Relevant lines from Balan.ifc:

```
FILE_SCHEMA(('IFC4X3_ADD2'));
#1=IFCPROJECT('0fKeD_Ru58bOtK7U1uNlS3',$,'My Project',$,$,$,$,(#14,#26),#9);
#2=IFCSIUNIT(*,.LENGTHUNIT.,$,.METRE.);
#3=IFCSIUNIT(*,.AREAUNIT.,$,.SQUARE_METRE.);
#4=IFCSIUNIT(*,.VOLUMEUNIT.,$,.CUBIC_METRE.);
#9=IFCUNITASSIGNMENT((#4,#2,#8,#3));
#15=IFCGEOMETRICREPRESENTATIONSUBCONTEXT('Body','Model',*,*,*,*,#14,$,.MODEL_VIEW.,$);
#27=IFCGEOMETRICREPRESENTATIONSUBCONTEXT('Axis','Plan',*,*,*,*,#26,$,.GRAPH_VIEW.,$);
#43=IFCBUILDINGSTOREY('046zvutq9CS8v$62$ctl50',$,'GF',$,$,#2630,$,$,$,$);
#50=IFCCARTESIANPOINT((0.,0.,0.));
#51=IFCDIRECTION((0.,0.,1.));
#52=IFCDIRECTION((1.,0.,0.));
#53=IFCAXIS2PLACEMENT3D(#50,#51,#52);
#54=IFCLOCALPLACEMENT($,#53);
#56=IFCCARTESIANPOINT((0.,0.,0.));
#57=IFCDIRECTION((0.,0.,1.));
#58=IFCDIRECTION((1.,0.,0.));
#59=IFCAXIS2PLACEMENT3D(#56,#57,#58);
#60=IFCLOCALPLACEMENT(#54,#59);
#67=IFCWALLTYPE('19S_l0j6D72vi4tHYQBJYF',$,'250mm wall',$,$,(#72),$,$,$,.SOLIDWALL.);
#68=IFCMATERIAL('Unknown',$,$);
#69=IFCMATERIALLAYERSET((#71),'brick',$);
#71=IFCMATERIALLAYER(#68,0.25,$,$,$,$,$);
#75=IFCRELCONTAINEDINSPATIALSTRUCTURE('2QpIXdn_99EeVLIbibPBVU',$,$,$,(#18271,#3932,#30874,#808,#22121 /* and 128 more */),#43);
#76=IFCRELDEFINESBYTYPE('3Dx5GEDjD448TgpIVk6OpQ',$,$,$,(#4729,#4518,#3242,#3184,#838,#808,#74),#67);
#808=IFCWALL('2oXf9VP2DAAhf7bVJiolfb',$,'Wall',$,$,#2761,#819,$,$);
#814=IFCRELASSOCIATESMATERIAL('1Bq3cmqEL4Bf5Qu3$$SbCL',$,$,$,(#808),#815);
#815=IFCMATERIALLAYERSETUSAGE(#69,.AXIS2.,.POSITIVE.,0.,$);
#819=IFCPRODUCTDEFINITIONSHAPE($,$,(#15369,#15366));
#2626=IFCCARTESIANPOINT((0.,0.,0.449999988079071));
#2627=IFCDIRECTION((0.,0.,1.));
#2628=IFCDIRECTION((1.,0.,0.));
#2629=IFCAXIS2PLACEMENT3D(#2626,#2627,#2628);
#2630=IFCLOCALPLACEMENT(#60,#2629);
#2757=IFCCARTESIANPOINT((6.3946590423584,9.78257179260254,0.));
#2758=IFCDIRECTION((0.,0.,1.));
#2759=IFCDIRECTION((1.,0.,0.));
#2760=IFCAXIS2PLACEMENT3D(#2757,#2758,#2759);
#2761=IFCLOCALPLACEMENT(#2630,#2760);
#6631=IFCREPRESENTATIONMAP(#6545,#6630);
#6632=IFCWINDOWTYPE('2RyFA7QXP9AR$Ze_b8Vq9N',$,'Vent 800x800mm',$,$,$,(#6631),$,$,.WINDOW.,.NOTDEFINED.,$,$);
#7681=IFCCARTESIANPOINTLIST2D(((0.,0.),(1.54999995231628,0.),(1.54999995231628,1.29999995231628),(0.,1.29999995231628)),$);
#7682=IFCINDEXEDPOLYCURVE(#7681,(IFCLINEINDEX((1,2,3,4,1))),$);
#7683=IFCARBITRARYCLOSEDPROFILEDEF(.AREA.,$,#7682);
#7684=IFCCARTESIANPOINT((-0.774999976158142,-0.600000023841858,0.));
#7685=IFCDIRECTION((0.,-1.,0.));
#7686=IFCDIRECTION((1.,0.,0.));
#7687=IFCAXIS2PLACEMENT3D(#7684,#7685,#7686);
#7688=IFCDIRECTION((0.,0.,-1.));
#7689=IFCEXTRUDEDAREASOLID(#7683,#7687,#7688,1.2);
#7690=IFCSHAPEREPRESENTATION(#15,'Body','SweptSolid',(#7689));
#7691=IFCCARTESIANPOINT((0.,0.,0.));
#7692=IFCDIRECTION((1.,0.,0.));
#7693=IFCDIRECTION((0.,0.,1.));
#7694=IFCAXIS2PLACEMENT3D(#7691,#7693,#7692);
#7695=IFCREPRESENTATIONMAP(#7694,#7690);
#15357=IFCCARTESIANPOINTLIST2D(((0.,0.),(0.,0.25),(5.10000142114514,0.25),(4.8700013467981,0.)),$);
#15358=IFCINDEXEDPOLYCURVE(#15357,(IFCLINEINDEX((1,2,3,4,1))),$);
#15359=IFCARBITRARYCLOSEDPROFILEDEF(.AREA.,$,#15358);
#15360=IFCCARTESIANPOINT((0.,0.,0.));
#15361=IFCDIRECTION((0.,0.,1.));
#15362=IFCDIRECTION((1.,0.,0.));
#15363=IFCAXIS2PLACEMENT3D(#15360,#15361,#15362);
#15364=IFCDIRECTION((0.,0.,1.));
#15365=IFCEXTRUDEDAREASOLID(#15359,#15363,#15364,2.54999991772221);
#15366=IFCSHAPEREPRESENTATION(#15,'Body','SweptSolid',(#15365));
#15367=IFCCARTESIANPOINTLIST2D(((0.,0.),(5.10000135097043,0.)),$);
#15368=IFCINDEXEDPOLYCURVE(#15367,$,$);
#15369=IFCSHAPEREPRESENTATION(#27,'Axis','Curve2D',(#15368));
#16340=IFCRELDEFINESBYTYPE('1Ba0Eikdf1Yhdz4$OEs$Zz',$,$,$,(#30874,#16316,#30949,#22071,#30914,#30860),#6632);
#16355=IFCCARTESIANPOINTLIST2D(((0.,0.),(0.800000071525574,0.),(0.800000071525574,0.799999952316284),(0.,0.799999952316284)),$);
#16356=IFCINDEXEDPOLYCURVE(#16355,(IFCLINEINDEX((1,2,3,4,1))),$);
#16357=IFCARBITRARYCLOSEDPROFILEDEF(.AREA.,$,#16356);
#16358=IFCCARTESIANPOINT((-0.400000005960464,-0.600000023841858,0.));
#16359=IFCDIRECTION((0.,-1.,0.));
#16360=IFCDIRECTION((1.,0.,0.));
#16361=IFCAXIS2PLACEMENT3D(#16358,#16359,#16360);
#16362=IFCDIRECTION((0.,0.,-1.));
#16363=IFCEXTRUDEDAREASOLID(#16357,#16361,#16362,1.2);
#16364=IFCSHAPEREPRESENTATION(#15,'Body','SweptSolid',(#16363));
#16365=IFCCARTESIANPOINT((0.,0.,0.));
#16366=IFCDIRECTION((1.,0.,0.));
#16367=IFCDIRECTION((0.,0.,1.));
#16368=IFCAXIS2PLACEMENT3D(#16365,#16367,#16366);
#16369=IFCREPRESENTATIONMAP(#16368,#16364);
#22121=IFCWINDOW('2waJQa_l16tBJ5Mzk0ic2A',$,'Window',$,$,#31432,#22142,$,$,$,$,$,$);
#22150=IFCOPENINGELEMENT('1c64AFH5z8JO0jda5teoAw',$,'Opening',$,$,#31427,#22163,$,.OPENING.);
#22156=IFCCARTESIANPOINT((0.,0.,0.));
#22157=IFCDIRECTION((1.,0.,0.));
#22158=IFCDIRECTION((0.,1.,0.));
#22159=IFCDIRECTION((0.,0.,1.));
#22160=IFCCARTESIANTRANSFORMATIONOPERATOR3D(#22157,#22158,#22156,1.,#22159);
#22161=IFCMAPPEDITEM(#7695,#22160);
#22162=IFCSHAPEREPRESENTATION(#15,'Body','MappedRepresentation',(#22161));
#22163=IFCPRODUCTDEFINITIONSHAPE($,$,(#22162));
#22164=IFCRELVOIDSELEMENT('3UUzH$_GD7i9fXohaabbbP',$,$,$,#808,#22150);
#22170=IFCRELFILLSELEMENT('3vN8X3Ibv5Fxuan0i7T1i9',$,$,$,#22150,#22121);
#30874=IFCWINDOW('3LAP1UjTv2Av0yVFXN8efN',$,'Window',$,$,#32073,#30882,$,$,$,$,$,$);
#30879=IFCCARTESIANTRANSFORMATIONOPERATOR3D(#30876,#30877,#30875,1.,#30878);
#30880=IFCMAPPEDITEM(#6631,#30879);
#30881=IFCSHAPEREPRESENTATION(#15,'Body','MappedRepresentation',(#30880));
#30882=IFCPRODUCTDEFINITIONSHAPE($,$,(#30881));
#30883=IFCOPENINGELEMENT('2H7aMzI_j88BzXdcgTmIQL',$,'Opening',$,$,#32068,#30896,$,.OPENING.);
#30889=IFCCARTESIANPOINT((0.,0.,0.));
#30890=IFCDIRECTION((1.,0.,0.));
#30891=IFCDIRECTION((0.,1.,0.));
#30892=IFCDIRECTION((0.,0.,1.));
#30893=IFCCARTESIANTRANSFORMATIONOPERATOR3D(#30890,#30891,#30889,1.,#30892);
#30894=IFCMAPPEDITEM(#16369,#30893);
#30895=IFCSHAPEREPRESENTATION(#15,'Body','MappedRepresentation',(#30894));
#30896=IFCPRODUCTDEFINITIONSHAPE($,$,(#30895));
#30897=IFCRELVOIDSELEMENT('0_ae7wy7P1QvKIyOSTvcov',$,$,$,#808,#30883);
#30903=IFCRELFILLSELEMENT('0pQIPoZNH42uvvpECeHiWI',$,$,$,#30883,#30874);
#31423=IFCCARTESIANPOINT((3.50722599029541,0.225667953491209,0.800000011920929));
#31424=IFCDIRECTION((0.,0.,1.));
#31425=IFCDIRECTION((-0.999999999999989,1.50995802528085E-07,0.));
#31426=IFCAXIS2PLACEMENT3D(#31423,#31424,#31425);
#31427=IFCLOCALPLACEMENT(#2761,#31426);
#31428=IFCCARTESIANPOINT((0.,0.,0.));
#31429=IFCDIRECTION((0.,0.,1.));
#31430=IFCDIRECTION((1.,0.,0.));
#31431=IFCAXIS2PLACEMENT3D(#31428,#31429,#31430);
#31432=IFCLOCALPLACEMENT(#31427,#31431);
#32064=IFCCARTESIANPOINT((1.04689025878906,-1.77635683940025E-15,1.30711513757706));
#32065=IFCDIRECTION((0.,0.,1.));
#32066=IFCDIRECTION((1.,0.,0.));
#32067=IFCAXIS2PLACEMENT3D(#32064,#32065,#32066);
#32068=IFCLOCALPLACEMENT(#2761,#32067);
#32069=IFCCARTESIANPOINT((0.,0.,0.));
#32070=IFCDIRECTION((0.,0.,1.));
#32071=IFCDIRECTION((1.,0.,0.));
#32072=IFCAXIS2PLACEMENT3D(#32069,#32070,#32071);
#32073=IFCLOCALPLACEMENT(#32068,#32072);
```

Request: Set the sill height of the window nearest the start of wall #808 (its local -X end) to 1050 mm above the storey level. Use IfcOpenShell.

```python
import numpy as np
import ifcopenshell
import ifcopenshell.api.geometry
import ifcopenshell.geom
import ifcopenshell.util.element
import ifcopenshell.util.placement
import ifcopenshell.util.shape
import ifcopenshell.util.unit

model = ifcopenshell.open("Balan.ifc")
unit_scale = ifcopenshell.util.unit.calculate_unit_scale(model)

window = model.by_guid("3LAP1UjTv2Av0yVFXN8efN")
opening = window.FillsVoids[0].RelatingOpeningElement
storey = ifcopenshell.util.element.get_container(window, ifc_class="IfcBuildingStorey")
level = ifcopenshell.util.placement.get_local_placement(storey.ObjectPlacement)[2, 3]

# The opening's origin need not be at the sill, so measure its lowest point.
shape = ifcopenshell.geom.create_shape(ifcopenshell.geom.settings(), opening)
bottom = ifcopenshell.util.shape.get_shape_bottom_elevation(shape, shape.geometry) / unit_scale
dz = level + 1.05 - bottom

shift = np.array([0.0, 0.0, dz])
# The window is placed relative to its opening, so it follows when the opening moves.
matrix = ifcopenshell.util.placement.get_local_placement(opening.ObjectPlacement)
matrix[:3, 3] += shift
ifcopenshell.api.geometry.edit_object_placement(
    model, product=opening, matrix=matrix, is_si=False, should_transform_children=True
)

print(f"moved by {dz * unit_scale:+.3f} m")

model.write("Balan_updated.ifc")
```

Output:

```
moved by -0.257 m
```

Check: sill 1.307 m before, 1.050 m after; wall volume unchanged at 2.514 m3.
